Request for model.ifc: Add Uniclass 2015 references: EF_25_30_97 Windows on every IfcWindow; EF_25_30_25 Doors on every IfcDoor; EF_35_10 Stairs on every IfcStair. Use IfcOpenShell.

First a look at what the model holds.

```python
import ifcopenshell

model = ifcopenshell.open("model.ifc")
print(model.schema)
print("classifications:", [c.Name for c in model.by_type("IfcClassification")])
for ifc_class in ("IfcDoor", "IfcRoof", "IfcStair", "IfcWall", "IfcWindow"):
    print(ifc_class, len(model.by_type(ifc_class)))
```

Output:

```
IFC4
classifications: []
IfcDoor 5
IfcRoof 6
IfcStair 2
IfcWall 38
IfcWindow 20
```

```python
import ifcopenshell
import ifcopenshell.api.classification

model = ifcopenshell.open("model.ifc")

system = ifcopenshell.api.classification.add_classification(model, classification="Uniclass 2015")

codes = {
    "IfcWindow": ("EF_25_30_97", "Windows"),
    "IfcDoor": ("EF_25_30_25", "Doors"),
    "IfcStair": ("EF_35_10", "Stairs"),
}
for ifc_class, (code, name) in codes.items():
    products = model.by_type(ifc_class)
    ifcopenshell.api.classification.add_reference(
        model, products=products, classification=system, identification=code, name=name
    )
    print(code, len(products))

model.write("model_edited.ifc")
```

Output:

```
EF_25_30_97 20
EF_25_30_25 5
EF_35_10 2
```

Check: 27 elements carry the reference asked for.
